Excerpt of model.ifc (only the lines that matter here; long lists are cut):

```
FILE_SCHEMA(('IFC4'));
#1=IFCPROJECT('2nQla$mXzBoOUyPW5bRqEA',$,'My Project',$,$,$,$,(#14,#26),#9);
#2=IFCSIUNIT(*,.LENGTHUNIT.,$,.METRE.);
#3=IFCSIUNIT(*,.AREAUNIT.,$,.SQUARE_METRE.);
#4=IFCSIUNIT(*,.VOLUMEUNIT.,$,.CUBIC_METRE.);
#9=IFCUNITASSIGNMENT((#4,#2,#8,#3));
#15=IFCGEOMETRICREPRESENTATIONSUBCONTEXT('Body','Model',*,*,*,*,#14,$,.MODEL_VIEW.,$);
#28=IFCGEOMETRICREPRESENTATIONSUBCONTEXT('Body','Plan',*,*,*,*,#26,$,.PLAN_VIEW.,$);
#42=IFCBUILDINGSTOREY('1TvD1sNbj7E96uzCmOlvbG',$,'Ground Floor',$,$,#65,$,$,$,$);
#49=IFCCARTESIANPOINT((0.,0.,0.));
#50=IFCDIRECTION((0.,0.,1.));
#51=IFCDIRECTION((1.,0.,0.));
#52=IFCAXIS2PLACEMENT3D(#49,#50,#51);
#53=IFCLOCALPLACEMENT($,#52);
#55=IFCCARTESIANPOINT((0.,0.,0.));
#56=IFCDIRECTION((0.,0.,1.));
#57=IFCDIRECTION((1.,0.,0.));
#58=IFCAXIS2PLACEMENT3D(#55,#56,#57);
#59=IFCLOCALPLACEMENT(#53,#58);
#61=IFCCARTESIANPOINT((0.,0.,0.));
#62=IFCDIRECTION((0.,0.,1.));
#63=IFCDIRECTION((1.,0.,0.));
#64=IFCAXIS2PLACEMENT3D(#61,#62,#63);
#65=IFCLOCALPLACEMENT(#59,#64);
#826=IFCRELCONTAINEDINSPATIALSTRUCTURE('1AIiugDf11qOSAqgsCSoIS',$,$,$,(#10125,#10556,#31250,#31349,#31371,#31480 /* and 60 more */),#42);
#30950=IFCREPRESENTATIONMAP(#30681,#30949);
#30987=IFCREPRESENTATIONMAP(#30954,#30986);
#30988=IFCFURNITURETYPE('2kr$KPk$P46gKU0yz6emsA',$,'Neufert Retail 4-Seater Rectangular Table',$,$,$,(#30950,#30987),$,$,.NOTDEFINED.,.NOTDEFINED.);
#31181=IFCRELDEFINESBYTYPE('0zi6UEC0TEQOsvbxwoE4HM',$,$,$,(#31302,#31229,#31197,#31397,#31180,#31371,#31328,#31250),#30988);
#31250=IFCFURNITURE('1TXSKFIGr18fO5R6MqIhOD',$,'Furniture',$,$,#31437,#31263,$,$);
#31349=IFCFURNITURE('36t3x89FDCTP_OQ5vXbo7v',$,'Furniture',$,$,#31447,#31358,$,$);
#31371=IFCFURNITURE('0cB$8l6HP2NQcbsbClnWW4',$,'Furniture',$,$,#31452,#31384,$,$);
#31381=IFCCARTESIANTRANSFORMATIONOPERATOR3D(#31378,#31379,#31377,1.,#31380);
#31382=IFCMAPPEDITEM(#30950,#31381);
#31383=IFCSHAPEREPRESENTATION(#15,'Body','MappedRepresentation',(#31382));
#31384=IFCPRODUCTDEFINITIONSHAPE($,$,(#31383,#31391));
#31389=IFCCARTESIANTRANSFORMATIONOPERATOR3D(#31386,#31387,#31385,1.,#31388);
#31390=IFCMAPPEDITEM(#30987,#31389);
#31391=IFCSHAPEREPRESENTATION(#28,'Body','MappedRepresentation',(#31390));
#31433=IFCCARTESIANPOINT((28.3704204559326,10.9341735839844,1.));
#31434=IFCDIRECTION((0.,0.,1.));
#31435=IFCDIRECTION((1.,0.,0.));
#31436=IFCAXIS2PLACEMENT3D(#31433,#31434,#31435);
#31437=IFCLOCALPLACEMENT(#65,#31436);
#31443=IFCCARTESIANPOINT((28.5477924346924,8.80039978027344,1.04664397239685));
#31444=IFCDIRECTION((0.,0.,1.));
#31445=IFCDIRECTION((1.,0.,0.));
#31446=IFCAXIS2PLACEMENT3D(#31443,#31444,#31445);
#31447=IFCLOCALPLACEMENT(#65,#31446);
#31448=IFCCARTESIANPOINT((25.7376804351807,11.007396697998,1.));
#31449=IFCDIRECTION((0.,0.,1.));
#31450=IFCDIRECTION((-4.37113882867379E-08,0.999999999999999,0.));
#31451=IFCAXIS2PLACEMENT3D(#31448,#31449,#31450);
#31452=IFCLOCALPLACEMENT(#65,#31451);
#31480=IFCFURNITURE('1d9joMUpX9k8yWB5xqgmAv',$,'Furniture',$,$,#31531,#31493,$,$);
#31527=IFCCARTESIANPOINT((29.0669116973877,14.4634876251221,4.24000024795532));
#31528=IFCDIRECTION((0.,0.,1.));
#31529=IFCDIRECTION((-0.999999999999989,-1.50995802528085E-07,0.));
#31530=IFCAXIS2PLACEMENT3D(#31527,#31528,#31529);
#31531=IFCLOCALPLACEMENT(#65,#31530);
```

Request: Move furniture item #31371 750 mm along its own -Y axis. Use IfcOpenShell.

```python
import ifcopenshell
import ifcopenshell.api.geometry
import ifcopenshell.util.placement

model = ifcopenshell.open("model.ifc")

item = model.by_guid("0cB$8l6HP2NQcbsbClnWW4")
matrix = ifcopenshell.util.placement.get_local_placement(item.ObjectPlacement)
matrix[:3, 3] -= matrix[:3, 1] * 0.75
ifcopenshell.api.geometry.edit_object_placement(model, product=item, matrix=matrix, is_si=False)

print(ifcopenshell.util.placement.get_local_placement(item.ObjectPlacement).round(3) + 0.0)

model.write("model_rev.ifc")
```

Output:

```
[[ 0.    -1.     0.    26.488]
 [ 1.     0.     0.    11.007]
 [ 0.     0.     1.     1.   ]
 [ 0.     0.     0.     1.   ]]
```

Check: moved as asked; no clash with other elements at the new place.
